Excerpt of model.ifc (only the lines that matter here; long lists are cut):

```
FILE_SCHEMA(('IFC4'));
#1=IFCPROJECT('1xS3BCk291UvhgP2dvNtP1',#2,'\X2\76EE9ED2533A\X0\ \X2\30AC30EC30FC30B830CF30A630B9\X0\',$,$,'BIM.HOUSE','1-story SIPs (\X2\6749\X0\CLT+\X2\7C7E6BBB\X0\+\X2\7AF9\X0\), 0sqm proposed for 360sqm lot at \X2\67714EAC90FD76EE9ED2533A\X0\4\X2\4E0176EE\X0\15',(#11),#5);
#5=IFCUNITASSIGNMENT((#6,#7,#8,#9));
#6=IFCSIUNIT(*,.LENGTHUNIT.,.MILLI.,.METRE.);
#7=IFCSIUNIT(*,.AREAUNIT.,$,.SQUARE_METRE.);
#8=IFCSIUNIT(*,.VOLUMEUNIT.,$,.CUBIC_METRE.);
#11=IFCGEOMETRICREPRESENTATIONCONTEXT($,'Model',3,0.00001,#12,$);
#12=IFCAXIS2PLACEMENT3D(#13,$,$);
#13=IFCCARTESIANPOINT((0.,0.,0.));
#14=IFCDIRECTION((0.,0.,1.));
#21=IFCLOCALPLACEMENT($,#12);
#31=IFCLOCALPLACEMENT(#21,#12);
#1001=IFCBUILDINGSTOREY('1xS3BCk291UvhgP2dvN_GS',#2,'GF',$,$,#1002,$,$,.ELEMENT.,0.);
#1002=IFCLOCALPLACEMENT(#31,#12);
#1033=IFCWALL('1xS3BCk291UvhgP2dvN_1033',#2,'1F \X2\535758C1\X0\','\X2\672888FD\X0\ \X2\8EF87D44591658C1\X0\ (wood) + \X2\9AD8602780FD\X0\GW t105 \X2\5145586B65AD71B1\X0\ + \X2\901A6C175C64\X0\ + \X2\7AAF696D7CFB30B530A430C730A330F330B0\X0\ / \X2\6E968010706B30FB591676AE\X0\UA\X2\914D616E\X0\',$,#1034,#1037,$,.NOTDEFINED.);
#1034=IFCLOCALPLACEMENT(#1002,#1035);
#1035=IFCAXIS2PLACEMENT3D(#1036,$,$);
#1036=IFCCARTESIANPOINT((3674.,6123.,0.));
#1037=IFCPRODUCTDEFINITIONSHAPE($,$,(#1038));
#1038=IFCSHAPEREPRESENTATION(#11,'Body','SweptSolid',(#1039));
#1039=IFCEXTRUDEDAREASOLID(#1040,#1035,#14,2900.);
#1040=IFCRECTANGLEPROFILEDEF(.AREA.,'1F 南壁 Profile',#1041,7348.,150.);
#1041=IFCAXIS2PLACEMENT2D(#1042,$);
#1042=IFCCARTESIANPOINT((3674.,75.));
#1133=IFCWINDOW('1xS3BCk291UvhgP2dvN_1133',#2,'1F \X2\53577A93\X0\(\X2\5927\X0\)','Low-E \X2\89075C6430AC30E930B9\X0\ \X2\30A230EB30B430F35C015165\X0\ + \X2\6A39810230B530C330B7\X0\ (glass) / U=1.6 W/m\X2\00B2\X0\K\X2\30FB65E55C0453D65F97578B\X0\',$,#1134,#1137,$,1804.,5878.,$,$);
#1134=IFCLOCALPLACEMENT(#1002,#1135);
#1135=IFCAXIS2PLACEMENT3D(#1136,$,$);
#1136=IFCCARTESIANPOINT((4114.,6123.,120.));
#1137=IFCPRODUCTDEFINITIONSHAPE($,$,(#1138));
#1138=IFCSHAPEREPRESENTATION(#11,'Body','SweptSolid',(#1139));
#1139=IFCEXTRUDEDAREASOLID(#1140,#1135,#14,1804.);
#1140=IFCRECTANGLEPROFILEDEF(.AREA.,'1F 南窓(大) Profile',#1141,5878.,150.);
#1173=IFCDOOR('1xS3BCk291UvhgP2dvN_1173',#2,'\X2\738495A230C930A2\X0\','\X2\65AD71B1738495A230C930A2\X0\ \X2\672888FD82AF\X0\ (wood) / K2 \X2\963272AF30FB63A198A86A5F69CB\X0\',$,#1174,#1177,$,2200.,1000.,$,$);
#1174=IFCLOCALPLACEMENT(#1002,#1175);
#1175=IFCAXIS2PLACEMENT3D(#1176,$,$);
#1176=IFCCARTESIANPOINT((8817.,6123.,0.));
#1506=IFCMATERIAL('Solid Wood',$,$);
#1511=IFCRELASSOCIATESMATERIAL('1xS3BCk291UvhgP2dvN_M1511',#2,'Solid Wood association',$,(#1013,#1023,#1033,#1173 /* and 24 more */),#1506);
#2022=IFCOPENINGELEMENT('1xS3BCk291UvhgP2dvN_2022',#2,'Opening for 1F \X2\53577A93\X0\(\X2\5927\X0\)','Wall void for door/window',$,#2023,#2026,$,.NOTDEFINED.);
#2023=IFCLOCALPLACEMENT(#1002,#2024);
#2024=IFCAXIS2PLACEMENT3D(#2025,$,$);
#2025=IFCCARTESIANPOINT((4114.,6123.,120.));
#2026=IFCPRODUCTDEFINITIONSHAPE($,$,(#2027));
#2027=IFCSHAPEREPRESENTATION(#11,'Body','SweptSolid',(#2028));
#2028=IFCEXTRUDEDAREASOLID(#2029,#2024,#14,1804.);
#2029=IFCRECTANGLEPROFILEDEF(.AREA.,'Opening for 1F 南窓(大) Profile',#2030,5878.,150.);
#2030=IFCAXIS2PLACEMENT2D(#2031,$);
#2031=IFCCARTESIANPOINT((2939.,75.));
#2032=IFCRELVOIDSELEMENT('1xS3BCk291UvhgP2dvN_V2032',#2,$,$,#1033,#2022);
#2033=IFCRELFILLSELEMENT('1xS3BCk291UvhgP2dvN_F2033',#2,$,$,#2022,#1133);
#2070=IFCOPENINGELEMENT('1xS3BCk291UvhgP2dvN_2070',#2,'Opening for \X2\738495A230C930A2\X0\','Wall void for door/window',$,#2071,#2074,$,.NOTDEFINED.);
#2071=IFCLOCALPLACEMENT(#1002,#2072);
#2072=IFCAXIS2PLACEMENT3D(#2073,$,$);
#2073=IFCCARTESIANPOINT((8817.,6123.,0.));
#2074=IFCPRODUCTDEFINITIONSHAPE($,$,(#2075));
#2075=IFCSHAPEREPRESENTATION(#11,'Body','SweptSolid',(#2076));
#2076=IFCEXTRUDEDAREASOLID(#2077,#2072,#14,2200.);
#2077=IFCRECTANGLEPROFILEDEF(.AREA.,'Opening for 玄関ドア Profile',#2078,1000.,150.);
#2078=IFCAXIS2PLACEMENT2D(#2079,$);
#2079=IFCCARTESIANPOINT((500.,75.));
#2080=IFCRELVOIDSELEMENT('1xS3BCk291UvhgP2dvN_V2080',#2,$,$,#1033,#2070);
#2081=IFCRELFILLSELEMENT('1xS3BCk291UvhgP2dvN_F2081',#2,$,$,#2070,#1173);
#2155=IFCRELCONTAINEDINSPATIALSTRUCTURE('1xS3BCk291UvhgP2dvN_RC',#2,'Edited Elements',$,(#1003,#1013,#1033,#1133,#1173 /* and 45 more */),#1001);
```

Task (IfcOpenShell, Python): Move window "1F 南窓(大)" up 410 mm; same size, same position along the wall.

```python
import numpy as np
import ifcopenshell
import ifcopenshell.api.geometry
import ifcopenshell.util.placement
import ifcopenshell.util.unit

model = ifcopenshell.open("model.ifc")
unit_scale = ifcopenshell.util.unit.calculate_unit_scale(model)

window = model.by_guid("1xS3BCk291UvhgP2dvN_1133")
opening = window.FillsVoids[0].RelatingOpeningElement
dz = 410.0

shift = np.array([0.0, 0.0, dz])
# The window is not placed relative to its opening, so move both.
for product in (opening, window):
    matrix = ifcopenshell.util.placement.get_local_placement(product.ObjectPlacement)
    matrix[:3, 3] += shift
    ifcopenshell.api.geometry.edit_object_placement(model, product=product, matrix=matrix, is_si=False)

print(f"moved by {dz * unit_scale:+.3f} m")

model.write("model_rev.ifc")
```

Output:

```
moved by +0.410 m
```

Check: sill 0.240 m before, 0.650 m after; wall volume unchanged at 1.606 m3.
